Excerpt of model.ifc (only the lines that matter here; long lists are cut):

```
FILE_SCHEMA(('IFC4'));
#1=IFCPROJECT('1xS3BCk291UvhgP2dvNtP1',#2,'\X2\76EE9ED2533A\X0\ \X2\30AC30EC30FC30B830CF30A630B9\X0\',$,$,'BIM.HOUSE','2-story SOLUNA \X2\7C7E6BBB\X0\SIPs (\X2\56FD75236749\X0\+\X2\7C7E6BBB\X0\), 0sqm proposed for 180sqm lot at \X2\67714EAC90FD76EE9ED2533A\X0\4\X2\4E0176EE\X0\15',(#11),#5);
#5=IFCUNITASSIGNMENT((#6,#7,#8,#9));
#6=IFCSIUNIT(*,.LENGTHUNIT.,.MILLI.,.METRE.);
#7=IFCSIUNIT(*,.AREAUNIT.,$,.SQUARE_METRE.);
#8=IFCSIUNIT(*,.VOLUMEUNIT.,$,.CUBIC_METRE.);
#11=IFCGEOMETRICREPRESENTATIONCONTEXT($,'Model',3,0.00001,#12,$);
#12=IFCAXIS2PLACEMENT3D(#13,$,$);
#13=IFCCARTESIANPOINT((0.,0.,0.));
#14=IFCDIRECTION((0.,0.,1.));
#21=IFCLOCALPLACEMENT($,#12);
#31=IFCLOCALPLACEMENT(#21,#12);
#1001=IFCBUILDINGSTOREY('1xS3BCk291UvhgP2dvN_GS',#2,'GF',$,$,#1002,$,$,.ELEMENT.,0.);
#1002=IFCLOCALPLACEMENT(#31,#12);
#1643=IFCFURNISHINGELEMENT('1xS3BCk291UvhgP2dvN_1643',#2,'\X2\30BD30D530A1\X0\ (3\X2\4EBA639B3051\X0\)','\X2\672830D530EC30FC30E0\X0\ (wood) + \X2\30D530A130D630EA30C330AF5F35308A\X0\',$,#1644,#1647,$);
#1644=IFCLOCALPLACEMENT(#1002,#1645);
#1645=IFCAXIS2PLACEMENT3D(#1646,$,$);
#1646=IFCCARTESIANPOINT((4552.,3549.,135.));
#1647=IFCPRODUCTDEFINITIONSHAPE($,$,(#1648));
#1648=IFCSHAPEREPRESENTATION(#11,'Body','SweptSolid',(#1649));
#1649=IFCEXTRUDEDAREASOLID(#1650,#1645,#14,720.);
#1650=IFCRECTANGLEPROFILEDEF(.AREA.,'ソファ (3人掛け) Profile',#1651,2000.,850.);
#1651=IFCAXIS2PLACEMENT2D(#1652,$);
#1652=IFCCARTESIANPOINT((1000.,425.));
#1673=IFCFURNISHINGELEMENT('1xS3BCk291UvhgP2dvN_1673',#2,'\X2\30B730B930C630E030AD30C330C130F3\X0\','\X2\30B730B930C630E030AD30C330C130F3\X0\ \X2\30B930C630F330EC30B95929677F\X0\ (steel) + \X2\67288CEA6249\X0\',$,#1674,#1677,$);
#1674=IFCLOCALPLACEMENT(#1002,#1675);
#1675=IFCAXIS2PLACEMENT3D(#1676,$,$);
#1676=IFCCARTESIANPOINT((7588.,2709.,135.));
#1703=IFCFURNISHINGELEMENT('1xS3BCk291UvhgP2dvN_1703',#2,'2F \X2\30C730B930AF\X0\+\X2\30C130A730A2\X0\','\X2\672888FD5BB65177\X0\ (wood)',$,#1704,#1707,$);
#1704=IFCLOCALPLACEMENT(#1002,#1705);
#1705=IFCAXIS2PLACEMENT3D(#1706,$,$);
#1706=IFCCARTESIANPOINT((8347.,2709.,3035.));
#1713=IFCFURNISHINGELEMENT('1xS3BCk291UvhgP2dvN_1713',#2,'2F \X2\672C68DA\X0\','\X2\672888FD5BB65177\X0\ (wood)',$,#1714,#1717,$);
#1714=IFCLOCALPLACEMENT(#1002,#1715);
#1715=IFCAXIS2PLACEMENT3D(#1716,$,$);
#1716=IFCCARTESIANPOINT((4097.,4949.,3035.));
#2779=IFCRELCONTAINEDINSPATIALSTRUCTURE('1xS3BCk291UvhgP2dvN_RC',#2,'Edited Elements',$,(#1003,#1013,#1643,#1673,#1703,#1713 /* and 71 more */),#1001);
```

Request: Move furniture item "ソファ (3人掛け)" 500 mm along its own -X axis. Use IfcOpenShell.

```python
import ifcopenshell
import ifcopenshell.api.geometry
import ifcopenshell.util.placement
import ifcopenshell.util.unit

model = ifcopenshell.open("model.ifc")
unit_scale = ifcopenshell.util.unit.calculate_unit_scale(model)

item = model.by_guid("1xS3BCk291UvhgP2dvN_1643")
matrix = ifcopenshell.util.placement.get_local_placement(item.ObjectPlacement)
matrix[:3, 3] -= matrix[:3, 0] * 0.5 / unit_scale
ifcopenshell.api.geometry.edit_object_placement(model, product=item, matrix=matrix, is_si=False)

print(ifcopenshell.util.placement.get_local_placement(item.ObjectPlacement).round(3) + 0.0)

model.write("model_edited.ifc")
```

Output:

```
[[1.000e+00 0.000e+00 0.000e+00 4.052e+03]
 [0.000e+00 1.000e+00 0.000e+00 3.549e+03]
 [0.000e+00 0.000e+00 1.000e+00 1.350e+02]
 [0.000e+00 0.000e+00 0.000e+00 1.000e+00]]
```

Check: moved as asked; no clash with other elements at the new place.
